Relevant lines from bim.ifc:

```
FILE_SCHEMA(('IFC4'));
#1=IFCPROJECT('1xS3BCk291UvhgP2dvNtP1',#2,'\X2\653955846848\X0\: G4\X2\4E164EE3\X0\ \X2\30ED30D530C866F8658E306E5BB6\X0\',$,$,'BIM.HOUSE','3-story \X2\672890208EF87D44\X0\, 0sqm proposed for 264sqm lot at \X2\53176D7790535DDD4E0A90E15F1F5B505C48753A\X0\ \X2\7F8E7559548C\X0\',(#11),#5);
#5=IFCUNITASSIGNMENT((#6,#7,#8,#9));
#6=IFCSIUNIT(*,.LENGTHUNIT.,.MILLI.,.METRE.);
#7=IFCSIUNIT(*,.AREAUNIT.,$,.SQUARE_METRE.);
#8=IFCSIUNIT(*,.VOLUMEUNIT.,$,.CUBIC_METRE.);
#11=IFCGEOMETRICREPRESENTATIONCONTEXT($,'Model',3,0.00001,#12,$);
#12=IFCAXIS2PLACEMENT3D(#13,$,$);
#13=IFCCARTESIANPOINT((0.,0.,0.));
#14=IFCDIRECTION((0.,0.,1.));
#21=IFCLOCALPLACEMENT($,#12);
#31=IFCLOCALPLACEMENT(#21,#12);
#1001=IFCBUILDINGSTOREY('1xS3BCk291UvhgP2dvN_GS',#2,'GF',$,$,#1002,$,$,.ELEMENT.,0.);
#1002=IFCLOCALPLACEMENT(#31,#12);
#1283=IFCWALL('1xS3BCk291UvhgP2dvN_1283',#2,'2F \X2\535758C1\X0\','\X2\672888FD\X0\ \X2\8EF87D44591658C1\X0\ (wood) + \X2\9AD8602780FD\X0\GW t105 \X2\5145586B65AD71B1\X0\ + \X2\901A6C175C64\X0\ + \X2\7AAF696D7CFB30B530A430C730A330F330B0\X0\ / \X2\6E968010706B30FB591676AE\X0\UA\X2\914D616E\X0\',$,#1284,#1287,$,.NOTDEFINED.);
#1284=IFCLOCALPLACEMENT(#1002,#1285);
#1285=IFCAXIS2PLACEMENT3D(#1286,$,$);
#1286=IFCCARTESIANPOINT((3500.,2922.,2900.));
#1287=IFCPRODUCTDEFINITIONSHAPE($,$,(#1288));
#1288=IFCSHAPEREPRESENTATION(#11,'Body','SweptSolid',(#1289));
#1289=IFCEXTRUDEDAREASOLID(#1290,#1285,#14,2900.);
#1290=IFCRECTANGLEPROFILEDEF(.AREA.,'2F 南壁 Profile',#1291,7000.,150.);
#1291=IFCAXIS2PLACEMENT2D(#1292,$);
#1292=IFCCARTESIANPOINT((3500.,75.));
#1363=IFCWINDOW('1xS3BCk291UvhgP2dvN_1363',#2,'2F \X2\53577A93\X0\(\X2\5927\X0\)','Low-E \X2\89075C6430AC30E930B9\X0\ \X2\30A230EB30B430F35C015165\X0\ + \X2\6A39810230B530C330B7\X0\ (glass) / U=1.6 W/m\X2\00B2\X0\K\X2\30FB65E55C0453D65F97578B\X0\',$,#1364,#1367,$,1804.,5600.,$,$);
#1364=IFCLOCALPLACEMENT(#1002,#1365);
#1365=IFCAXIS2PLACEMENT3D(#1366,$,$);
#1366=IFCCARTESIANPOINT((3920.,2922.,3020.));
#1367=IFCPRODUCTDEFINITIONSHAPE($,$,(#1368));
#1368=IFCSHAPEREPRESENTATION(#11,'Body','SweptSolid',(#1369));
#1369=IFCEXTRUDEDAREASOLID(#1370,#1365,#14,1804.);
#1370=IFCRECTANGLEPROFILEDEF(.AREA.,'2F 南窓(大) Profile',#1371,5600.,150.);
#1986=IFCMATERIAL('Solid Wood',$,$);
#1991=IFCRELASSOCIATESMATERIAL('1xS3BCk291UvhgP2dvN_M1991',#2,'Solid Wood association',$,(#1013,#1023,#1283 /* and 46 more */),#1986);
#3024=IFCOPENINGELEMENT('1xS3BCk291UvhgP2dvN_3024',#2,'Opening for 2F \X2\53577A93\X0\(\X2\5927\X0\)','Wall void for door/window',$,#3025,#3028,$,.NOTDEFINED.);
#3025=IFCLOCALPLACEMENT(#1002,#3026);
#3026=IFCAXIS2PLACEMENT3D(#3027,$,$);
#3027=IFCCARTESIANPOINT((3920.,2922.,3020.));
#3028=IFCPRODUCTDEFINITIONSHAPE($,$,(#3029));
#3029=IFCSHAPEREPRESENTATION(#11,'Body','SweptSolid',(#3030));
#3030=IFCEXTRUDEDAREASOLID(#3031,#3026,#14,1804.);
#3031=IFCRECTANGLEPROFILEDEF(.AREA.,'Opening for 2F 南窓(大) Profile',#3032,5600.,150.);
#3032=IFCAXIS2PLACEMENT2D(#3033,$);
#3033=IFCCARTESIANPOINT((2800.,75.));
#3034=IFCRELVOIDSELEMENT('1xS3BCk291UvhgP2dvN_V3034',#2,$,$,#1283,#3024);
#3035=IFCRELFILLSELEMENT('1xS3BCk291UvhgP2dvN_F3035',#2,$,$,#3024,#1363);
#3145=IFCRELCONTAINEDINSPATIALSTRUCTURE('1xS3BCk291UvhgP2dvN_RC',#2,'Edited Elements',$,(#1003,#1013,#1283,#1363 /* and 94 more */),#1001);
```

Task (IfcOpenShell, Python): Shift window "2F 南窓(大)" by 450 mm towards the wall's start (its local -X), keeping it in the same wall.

```python
import ifcopenshell
import ifcopenshell.api.geometry
import ifcopenshell.util.placement

model = ifcopenshell.open("bim.ifc")

window = model.by_guid("1xS3BCk291UvhgP2dvN_1363")
opening = window.FillsVoids[0].RelatingOpeningElement
wall = opening.VoidsElements[0].RelatingBuildingElement

wall_matrix = ifcopenshell.util.placement.get_local_placement(wall.ObjectPlacement)
shift = wall_matrix[:3, 0] * -450.0
before = ifcopenshell.util.placement.get_local_placement(window.ObjectPlacement)[:3, 3].copy()

# The window is not placed relative to its opening, so move both.
for product in (opening, window):
    matrix = ifcopenshell.util.placement.get_local_placement(product.ObjectPlacement)
    matrix[:3, 3] += shift
    ifcopenshell.api.geometry.edit_object_placement(model, product=product, matrix=matrix, is_si=False)

after = ifcopenshell.util.placement.get_local_placement(window.ObjectPlacement)[:3, 3]
print("window moved by", (after - before).round(3) + 0.0)

model.write("bim-out.ifc")
```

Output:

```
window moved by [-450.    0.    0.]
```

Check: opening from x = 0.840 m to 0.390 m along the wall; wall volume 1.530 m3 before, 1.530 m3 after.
